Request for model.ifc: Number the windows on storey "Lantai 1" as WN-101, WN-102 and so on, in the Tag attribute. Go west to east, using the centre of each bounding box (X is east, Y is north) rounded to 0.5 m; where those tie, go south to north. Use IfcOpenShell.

First a look at what the model holds.

```python
import ifcopenshell
import ifcopenshell.util.element
import ifcopenshell.util.placement

model = ifcopenshell.open("model.ifc")
print(model.schema)
storey = next(s for s in model.by_type("IfcBuildingStorey") if s.Name == "Lantai 1")
windows = [e for e in ifcopenshell.util.element.get_decomposition(storey) if e.is_a("IfcWindow")]
for e in sorted(windows, key=lambda e: e.id()):
    origin = ifcopenshell.util.placement.get_local_placement(e.ObjectPlacement)[:3, 3]
    print(e.id(), e.Tag, e.Name, origin.round(2) + 0.0, sep=" | ")
```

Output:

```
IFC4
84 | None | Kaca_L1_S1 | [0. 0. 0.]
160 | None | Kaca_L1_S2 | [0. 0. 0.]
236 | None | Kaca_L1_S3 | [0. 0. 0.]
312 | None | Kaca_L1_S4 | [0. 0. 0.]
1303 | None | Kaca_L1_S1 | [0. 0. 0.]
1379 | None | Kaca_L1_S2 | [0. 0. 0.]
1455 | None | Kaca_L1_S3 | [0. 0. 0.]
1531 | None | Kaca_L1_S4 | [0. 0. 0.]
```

```python
import ifcopenshell
import ifcopenshell.geom
import ifcopenshell.util.element
import ifcopenshell.util.shape

model = ifcopenshell.open("model.ifc")
settings = ifcopenshell.geom.settings()
settings.set("use-world-coords", True)


def centre(element):
    shape = ifcopenshell.geom.create_shape(settings, element)
    return ifcopenshell.util.shape.get_bbox_centroid(shape.geometry)


storey = next(s for s in model.by_type("IfcBuildingStorey") if s.Name == "Lantai 1")
windows = [e for e in ifcopenshell.util.element.get_decomposition(storey) if e.is_a("IfcWindow")]

# Insertion points can sit at a corner or the storey origin, so sort by the geometry (in metres).
centres = {e: centre(e) for e in windows}
windows.sort(key=lambda e: (round(centres[e][0] / 0.5), centres[e][1]))

for i, e in enumerate(windows, start=1):
    number = f"WN-1{i:02d}"
    e.Tag = number
    print(e.id(), number)

model.write("model-out.ifc")
```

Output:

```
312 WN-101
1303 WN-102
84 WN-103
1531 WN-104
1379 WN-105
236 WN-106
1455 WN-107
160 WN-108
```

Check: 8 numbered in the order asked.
